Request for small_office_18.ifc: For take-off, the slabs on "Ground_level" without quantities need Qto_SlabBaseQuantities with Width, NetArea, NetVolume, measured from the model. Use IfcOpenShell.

First a look at what the model holds.

```python
import ifcopenshell
import ifcopenshell.util.element
import ifcopenshell.util.unit

model = ifcopenshell.open("small_office_18.ifc")
print(model.schema)
for unit_type in ("LENGTHUNIT", "AREAUNIT", "VOLUMEUNIT"):
    print(unit_type, ifcopenshell.util.unit.calculate_unit_scale(model, unit_type))
storey = next(s for s in model.by_type("IfcBuildingStorey") if s.Name == "Ground_level")
slabs = [e for e in ifcopenshell.util.element.get_decomposition(storey) if e.is_a("IfcSlab")]
for e in sorted(slabs, key=lambda e: e.id()):
    print(e.id(), e.is_a(), e.Name, list(ifcopenshell.util.element.get_psets(e, qtos_only=True)), sep=" | ")
```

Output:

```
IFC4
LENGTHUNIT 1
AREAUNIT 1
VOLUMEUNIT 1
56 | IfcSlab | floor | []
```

```python
import ifcopenshell
import ifcopenshell.api.pset
import ifcopenshell.geom
import ifcopenshell.util.element
import ifcopenshell.util.shape
import ifcopenshell.util.unit

model = ifcopenshell.open("small_office_18.ifc")
unit_scale = ifcopenshell.util.unit.calculate_unit_scale(model)
area_scale = ifcopenshell.util.unit.calculate_unit_scale(model, "AREAUNIT")
volume_scale = ifcopenshell.util.unit.calculate_unit_scale(model, "VOLUMEUNIT")
settings = ifcopenshell.geom.settings()

storey = next(s for s in model.by_type("IfcBuildingStorey") if s.Name == "Ground_level")
slabs = [e for e in ifcopenshell.util.element.get_decomposition(storey) if e.is_a("IfcSlab")]

for e in sorted(slabs, key=lambda e: e.id()):
    if ifcopenshell.util.element.get_psets(e, qtos_only=True, should_inherit=False):
        continue
    # Geometry comes back in metres, in the element's own axes.
    shape = ifcopenshell.geom.create_shape(settings, e)
    values = {
        "Width": ifcopenshell.util.shape.get_z(shape.geometry) / unit_scale,
        "NetArea": ifcopenshell.util.shape.get_footprint_area(shape.geometry) / area_scale,
        "NetVolume": ifcopenshell.util.shape.get_volume(shape.geometry) / volume_scale,
    }
    qto = ifcopenshell.api.pset.add_qto(model, product=e, name="Qto_SlabBaseQuantities")
    ifcopenshell.api.pset.edit_qto(model, qto=qto, properties=values)
    print(e.id(), {k: round(v, 3) for k, v in values.items()})

model.write("small_office_18_updated.ifc")
```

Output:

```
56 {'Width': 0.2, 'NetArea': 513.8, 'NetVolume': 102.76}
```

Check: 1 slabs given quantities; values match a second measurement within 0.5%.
